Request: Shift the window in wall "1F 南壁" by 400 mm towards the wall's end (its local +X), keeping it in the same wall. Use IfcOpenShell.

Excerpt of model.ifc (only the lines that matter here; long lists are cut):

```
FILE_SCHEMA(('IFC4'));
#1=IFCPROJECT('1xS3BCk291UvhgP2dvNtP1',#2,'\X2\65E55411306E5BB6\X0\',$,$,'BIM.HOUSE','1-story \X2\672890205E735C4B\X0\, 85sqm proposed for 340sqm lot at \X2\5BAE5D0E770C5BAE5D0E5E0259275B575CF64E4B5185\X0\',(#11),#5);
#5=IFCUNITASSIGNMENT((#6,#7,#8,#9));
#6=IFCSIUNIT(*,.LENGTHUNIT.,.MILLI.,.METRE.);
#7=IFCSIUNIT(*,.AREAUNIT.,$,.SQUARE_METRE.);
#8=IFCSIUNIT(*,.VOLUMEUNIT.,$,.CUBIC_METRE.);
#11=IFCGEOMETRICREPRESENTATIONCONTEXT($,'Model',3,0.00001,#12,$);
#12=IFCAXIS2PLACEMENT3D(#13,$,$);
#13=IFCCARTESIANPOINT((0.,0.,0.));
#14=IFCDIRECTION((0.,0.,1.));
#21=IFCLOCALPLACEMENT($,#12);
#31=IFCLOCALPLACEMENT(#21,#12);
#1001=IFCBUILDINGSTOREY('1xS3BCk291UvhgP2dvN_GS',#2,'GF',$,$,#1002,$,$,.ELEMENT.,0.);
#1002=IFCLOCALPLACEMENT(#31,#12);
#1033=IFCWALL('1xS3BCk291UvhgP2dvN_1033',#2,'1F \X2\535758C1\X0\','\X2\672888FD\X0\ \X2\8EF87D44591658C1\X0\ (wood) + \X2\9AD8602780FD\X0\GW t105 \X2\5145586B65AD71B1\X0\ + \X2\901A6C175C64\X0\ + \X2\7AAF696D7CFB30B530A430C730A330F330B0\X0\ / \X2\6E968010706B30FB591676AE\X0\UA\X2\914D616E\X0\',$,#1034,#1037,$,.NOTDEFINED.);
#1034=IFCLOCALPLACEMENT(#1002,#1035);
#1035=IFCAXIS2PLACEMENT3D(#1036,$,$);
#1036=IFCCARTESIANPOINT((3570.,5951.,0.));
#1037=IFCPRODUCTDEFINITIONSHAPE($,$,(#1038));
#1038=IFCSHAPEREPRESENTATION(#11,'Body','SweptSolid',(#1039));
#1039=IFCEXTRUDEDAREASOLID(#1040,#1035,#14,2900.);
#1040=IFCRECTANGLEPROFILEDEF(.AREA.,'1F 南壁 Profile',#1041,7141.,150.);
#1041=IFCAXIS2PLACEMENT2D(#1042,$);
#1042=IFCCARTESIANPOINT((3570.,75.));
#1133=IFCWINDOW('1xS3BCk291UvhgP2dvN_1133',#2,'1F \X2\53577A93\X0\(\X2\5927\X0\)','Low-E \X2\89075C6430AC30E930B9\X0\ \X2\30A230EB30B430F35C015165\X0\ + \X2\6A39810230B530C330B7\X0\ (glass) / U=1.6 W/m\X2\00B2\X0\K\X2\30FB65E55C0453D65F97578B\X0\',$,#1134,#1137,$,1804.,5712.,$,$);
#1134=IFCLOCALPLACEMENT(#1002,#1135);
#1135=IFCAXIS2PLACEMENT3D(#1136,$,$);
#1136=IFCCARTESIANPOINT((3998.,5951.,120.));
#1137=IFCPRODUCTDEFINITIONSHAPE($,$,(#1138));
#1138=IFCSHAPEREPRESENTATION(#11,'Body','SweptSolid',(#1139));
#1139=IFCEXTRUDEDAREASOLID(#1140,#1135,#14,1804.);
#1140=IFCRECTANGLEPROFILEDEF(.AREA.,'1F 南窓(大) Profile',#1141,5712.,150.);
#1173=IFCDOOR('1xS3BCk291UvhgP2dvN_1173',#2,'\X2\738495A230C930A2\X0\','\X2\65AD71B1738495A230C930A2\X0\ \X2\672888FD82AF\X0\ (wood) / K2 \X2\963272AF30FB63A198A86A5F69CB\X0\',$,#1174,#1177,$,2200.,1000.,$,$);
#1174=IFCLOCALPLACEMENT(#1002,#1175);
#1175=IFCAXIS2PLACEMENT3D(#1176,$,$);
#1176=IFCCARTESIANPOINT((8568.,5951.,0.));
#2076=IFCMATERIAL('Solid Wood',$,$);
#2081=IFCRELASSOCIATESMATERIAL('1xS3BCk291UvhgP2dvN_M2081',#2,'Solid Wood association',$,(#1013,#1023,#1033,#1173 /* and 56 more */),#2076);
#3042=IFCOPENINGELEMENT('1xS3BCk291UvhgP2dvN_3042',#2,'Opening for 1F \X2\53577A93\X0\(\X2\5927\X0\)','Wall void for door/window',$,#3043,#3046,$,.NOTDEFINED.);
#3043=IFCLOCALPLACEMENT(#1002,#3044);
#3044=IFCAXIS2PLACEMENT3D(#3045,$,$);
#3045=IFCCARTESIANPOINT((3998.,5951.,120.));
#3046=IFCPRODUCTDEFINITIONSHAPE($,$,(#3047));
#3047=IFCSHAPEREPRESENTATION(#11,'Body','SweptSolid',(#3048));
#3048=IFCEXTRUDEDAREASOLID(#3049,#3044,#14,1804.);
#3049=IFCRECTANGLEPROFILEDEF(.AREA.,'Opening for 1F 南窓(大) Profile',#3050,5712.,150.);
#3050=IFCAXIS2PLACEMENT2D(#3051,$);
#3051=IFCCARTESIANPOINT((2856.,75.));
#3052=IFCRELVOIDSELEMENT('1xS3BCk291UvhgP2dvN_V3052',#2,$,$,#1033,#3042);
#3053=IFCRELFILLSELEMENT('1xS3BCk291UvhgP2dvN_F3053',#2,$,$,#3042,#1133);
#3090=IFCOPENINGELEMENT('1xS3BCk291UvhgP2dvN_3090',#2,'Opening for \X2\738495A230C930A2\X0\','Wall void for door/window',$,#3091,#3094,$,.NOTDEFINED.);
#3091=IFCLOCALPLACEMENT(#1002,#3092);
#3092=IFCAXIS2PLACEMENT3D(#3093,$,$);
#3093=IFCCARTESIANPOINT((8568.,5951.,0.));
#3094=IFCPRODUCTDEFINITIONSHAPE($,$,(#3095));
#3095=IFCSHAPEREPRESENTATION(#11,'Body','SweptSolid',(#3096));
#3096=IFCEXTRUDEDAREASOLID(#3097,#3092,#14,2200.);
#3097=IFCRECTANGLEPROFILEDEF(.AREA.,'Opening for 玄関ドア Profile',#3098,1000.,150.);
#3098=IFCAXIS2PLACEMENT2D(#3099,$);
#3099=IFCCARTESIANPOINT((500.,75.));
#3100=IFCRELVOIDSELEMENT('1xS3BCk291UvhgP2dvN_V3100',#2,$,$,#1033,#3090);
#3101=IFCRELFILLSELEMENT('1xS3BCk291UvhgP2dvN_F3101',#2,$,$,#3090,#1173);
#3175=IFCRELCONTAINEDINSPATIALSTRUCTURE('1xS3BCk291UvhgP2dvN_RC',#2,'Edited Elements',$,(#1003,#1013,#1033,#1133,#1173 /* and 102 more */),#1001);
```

```python
import ifcopenshell
import ifcopenshell.api.geometry
import ifcopenshell.util.placement
import ifcopenshell.util.unit

model = ifcopenshell.open("model.ifc")
unit_scale = ifcopenshell.util.unit.calculate_unit_scale(model)

window = model.by_guid("1xS3BCk291UvhgP2dvN_1133")
opening = window.FillsVoids[0].RelatingOpeningElement
wall = opening.VoidsElements[0].RelatingBuildingElement

wall_matrix = ifcopenshell.util.placement.get_local_placement(wall.ObjectPlacement)
shift = wall_matrix[:3, 0] * 0.4 / unit_scale
before = ifcopenshell.util.placement.get_local_placement(window.ObjectPlacement)[:3, 3].copy()

# The window is not placed relative to its opening, so move both.
for product in (opening, window):
    matrix = ifcopenshell.util.placement.get_local_placement(product.ObjectPlacement)
    matrix[:3, 3] += shift
    ifcopenshell.api.geometry.edit_object_placement(model, product=product, matrix=matrix, is_si=False)

after = ifcopenshell.util.placement.get_local_placement(window.ObjectPlacement)[:3, 3]
print("window moved by", (after - before).round(3) + 0.0)

model.write("model-out.ifc")
```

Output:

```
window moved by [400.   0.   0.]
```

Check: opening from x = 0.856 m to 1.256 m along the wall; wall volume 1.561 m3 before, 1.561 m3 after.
